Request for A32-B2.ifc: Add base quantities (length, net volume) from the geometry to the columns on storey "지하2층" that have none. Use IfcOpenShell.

First a look at what the model holds.

```python
import ifcopenshell
import ifcopenshell.util.element
import ifcopenshell.util.unit

model = ifcopenshell.open("A32-B2.ifc")
print(model.schema)
for unit_type in ("LENGTHUNIT", "AREAUNIT", "VOLUMEUNIT"):
    print(unit_type, ifcopenshell.util.unit.calculate_unit_scale(model, unit_type))
storey = next(s for s in model.by_type("IfcBuildingStorey") if s.Name == "지하2층")
columns = [e for e in ifcopenshell.util.element.get_decomposition(storey) if e.is_a("IfcColumn")]
for e in sorted(columns, key=lambda e: e.id()):
    print(e.id(), e.is_a(), e.Name, list(ifcopenshell.util.element.get_psets(e, qtos_only=True)), sep=" | ")
```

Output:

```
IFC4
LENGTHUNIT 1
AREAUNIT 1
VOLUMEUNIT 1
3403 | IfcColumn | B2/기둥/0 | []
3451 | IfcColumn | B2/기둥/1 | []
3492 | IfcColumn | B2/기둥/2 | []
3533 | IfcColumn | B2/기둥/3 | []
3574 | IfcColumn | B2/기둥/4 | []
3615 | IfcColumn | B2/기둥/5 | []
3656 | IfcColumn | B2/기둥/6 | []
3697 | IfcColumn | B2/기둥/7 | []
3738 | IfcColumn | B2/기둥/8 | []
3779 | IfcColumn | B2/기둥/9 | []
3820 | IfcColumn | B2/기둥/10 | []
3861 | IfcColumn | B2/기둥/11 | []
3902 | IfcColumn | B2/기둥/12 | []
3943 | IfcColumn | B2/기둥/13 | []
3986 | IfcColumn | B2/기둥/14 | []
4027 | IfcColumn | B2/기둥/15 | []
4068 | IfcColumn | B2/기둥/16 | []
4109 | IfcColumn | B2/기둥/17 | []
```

```python
import ifcopenshell
import ifcopenshell.api.pset
import ifcopenshell.geom
import ifcopenshell.util.element
import ifcopenshell.util.shape
import ifcopenshell.util.unit

model = ifcopenshell.open("A32-B2.ifc")
unit_scale = ifcopenshell.util.unit.calculate_unit_scale(model)
volume_scale = ifcopenshell.util.unit.calculate_unit_scale(model, "VOLUMEUNIT")
settings = ifcopenshell.geom.settings()

storey = next(s for s in model.by_type("IfcBuildingStorey") if s.Name == "지하2층")
columns = [e for e in ifcopenshell.util.element.get_decomposition(storey) if e.is_a("IfcColumn")]

for e in sorted(columns, key=lambda e: e.id()):
    if ifcopenshell.util.element.get_psets(e, qtos_only=True, should_inherit=False):
        continue
    # Geometry comes back in metres, in the element's own axes.
    shape = ifcopenshell.geom.create_shape(settings, e)
    values = {
        "Length": ifcopenshell.util.shape.get_z(shape.geometry) / unit_scale,
        "NetVolume": ifcopenshell.util.shape.get_volume(shape.geometry) / volume_scale,
    }
    qto = ifcopenshell.api.pset.add_qto(model, product=e, name="Qto_ColumnBaseQuantities")
    ifcopenshell.api.pset.edit_qto(model, qto=qto, properties=values)
    print(e.id(), {k: round(v, 3) for k, v in values.items()})

model.write("A32-B2_rev.ifc")
```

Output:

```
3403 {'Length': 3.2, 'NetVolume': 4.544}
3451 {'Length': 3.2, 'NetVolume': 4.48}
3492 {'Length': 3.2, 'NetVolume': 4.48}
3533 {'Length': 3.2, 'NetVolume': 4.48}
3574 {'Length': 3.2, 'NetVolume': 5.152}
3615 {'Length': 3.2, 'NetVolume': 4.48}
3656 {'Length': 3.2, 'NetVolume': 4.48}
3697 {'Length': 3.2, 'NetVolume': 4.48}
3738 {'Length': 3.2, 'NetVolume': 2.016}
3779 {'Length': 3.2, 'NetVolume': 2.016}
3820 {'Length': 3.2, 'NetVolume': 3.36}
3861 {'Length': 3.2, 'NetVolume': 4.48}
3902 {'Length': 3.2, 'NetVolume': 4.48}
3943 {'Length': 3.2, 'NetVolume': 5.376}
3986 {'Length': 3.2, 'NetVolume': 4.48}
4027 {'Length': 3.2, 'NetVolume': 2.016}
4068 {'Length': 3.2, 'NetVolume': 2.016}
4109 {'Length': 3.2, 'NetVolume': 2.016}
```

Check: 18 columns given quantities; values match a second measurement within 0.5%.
